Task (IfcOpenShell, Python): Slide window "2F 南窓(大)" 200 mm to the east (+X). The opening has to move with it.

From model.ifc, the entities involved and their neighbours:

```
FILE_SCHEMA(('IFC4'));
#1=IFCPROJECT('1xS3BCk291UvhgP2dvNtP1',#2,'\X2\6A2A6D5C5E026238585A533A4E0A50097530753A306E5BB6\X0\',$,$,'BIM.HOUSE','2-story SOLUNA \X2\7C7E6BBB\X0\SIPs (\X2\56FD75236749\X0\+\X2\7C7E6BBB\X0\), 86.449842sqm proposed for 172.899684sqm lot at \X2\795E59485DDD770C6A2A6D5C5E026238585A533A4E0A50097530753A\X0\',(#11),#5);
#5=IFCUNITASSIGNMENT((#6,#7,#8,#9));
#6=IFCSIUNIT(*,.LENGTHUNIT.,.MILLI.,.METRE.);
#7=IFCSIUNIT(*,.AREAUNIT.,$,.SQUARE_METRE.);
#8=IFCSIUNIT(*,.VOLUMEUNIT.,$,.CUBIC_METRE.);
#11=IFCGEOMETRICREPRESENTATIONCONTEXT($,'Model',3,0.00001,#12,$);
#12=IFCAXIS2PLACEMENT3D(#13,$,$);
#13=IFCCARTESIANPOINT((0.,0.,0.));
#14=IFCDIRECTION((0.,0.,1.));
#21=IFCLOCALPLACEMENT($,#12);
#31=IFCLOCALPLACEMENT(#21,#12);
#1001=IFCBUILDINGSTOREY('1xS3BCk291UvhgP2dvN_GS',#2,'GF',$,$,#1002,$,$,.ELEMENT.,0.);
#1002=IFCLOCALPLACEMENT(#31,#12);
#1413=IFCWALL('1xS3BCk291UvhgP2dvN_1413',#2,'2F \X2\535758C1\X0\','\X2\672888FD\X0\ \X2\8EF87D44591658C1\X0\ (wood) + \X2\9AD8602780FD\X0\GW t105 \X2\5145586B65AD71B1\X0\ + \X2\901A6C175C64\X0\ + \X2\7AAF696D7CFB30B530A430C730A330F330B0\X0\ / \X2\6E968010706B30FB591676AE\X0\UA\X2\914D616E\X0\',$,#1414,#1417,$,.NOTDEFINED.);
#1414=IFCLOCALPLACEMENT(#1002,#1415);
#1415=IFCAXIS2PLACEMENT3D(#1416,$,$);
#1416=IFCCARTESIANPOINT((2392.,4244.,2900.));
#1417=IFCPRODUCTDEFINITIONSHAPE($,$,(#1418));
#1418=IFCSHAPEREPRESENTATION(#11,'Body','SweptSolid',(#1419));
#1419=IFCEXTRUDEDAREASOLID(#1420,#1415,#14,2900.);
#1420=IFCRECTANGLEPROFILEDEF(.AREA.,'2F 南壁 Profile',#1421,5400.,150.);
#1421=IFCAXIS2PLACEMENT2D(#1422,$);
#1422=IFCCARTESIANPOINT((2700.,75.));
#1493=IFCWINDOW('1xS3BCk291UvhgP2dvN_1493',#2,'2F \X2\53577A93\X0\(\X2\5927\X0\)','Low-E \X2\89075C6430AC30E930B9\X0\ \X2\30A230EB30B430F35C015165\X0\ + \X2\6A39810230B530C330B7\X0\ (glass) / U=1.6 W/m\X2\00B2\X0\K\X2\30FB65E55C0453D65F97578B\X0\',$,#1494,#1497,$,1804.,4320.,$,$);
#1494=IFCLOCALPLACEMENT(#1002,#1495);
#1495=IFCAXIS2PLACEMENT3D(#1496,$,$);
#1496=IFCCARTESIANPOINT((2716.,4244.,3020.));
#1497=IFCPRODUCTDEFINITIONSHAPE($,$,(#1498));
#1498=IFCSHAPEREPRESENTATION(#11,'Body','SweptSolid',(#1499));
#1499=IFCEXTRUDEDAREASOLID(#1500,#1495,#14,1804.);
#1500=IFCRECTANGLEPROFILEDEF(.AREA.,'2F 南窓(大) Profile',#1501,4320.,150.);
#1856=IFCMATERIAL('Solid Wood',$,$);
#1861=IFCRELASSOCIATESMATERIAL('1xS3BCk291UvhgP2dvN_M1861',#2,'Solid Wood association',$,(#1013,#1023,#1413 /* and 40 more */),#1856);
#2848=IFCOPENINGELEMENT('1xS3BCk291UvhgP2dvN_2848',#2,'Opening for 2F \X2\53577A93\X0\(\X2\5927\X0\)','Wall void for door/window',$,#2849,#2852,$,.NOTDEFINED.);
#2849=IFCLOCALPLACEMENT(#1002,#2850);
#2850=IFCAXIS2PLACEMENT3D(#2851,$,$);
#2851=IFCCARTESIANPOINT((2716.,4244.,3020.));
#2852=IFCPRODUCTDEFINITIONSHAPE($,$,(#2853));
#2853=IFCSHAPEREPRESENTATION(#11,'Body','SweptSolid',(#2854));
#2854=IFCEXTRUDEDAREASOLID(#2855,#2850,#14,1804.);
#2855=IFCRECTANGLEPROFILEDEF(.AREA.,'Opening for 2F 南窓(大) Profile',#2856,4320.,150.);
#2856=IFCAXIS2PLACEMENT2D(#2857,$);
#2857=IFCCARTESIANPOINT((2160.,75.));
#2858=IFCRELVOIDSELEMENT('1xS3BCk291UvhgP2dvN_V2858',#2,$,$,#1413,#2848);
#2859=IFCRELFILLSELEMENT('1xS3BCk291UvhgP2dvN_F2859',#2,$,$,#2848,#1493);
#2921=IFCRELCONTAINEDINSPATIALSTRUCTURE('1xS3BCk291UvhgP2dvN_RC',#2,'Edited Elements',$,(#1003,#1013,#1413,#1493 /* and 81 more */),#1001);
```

```python
import ifcopenshell
import ifcopenshell.api.geometry
import ifcopenshell.util.placement
import ifcopenshell.util.unit

model = ifcopenshell.open("model.ifc")
unit_scale = ifcopenshell.util.unit.calculate_unit_scale(model)

window = model.by_guid("1xS3BCk291UvhgP2dvN_1493")
opening = window.FillsVoids[0].RelatingOpeningElement
wall = opening.VoidsElements[0].RelatingBuildingElement

wall_matrix = ifcopenshell.util.placement.get_local_placement(wall.ObjectPlacement)
shift = wall_matrix[:3, 0] * 0.2 / unit_scale
before = ifcopenshell.util.placement.get_local_placement(window.ObjectPlacement)[:3, 3].copy()

# The window is not placed relative to its opening, so move both.
for product in (opening, window):
    matrix = ifcopenshell.util.placement.get_local_placement(product.ObjectPlacement)
    matrix[:3, 3] += shift
    ifcopenshell.api.geometry.edit_object_placement(model, product=product, matrix=matrix, is_si=False)

after = ifcopenshell.util.placement.get_local_placement(window.ObjectPlacement)[:3, 3]
print("window moved by", (after - before).round(3) + 0.0)

model.write("model_v2.ifc")
```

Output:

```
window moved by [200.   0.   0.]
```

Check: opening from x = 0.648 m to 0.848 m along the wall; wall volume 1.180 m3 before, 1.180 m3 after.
